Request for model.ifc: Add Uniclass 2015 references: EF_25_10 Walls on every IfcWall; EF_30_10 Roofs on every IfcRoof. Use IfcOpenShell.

First a look at what the model holds.

```python
import ifcopenshell

model = ifcopenshell.open("model.ifc")
print(model.schema)
print("classifications:", [c.Name for c in model.by_type("IfcClassification")])
for ifc_class in ("IfcDoor", "IfcRoof", "IfcStair", "IfcWall", "IfcWindow"):
    print(ifc_class, len(model.by_type(ifc_class)))
```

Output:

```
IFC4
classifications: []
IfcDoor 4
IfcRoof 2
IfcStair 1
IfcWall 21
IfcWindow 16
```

```python
import ifcopenshell
import ifcopenshell.api.classification

model = ifcopenshell.open("model.ifc")

system = ifcopenshell.api.classification.add_classification(model, classification="Uniclass 2015")

codes = {
    "IfcWall": ("EF_25_10", "Walls"),
    "IfcRoof": ("EF_30_10", "Roofs"),
}
for ifc_class, (code, name) in codes.items():
    products = model.by_type(ifc_class)
    ifcopenshell.api.classification.add_reference(
        model, products=products, classification=system, identification=code, name=name
    )
    print(code, len(products))

model.write("model_rev.ifc")
```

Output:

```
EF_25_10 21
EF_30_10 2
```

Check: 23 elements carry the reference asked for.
